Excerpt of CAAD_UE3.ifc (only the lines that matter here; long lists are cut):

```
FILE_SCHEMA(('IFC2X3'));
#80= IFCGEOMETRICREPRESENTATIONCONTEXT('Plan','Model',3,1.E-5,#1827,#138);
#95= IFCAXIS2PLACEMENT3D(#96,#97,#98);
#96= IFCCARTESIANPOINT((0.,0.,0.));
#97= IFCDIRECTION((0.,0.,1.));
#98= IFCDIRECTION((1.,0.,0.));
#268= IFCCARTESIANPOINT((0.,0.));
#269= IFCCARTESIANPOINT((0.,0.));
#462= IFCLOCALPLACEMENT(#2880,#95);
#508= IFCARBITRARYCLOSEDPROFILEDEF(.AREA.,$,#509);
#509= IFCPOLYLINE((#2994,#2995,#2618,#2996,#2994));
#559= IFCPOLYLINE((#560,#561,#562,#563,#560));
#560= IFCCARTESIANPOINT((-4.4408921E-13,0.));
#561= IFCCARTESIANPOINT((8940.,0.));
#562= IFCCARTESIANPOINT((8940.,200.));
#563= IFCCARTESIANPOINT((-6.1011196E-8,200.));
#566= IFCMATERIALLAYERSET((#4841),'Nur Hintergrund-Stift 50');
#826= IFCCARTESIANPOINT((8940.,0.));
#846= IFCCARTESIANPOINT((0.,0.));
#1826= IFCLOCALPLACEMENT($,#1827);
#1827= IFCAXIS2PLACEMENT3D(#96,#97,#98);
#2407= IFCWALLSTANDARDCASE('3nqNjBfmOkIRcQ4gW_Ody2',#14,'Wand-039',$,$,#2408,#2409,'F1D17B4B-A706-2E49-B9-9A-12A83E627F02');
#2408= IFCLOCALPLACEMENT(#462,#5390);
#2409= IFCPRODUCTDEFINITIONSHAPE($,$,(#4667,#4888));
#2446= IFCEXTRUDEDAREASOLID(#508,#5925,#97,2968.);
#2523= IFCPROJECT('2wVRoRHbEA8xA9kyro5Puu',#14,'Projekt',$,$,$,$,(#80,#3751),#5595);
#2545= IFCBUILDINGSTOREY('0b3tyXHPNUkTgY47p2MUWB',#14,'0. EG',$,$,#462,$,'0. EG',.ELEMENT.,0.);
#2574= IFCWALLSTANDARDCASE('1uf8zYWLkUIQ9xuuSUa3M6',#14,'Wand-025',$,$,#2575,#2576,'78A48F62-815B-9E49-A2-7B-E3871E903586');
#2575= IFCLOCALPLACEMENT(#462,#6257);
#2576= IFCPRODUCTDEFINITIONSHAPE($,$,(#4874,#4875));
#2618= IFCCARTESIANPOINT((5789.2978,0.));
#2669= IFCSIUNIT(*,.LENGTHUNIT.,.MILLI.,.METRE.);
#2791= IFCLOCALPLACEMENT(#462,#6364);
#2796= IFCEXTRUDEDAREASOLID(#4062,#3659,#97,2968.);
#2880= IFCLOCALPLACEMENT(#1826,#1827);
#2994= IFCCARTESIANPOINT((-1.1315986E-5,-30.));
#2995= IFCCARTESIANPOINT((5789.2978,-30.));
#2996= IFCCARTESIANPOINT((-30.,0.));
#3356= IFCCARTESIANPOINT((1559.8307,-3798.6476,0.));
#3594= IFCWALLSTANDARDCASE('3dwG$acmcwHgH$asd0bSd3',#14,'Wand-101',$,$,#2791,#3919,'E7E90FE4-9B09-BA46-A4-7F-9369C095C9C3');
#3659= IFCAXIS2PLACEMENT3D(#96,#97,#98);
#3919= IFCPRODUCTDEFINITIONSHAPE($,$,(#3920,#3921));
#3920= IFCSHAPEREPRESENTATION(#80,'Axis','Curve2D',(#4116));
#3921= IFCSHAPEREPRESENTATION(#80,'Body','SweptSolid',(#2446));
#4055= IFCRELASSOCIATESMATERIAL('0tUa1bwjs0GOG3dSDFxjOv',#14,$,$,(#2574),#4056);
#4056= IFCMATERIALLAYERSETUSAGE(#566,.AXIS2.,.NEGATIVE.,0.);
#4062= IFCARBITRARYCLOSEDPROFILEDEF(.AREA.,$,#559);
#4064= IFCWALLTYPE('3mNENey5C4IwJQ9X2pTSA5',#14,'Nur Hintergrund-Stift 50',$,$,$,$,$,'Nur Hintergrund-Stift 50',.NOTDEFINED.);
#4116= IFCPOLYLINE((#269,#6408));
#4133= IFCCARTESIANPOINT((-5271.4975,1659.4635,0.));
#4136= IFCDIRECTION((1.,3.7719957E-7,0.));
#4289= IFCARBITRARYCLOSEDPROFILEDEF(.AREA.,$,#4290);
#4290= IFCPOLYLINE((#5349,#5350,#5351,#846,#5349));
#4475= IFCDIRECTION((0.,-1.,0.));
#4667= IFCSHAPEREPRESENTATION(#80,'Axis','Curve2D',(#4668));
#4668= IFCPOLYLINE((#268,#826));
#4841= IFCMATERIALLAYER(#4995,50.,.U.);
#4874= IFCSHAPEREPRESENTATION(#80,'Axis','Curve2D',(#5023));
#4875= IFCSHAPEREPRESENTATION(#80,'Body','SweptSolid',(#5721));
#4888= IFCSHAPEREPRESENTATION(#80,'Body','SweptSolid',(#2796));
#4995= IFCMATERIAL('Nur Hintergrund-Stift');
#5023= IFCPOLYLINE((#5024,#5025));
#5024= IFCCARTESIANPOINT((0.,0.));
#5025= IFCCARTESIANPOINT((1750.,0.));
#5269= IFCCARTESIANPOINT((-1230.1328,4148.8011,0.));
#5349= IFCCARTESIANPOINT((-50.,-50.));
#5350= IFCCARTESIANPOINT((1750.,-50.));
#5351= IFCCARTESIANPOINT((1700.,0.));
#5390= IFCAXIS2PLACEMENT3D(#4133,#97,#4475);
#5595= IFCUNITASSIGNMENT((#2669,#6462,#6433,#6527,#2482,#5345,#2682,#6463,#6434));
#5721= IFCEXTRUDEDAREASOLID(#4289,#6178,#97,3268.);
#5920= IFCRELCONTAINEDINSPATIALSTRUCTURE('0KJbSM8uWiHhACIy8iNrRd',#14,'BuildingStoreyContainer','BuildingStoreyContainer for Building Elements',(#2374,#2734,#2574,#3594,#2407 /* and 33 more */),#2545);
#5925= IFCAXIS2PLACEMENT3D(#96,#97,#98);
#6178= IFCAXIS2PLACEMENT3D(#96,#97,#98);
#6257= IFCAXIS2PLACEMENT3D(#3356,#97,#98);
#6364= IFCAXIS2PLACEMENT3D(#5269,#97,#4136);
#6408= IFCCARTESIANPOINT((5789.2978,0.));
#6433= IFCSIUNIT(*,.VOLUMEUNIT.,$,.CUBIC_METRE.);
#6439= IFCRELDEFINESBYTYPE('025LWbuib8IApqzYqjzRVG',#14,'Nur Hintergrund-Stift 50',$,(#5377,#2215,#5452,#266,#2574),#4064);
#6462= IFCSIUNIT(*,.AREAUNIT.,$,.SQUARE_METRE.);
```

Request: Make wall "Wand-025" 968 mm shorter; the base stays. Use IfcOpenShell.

```python
import ifcopenshell
import ifcopenshell.geom
import ifcopenshell.util.shape

model = ifcopenshell.open("CAAD_UE3.ifc")
settings = ifcopenshell.geom.settings()


def volume(element):
    """Net volume in cubic metres, openings subtracted."""
    shape = ifcopenshell.geom.create_shape(settings, element)
    return ifcopenshell.util.shape.get_volume(shape.geometry)


wall = model.by_guid("1uf8zYWLkUIQ9xuuSUa3M6")
before = volume(wall)

body = next(r for r in wall.Representation.Representations if r.RepresentationIdentifier == "Body")
solid = body.Items[0]
old_height = solid.Depth
solid.Depth -= 968.0
after = volume(wall)

print(f"height {old_height:g} -> {solid.Depth:g}, volume {before:.3f} -> {after:.3f} m3")

model.write("CAAD_UE3_edited.ifc")
```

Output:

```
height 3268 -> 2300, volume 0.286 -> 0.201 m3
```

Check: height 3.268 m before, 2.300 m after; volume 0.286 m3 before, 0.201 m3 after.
